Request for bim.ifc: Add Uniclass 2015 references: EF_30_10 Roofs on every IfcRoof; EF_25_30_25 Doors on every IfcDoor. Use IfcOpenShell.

First a look at what the model holds.

```python
import ifcopenshell

model = ifcopenshell.open("bim.ifc")
print(model.schema)
print("classifications:", [c.Name for c in model.by_type("IfcClassification")])
for ifc_class in ("IfcDoor", "IfcRoof", "IfcStair", "IfcWall", "IfcWindow"):
    print(ifc_class, len(model.by_type(ifc_class)))
```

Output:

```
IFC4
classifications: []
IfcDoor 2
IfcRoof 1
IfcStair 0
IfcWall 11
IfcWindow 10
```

```python
import ifcopenshell
import ifcopenshell.api.classification

model = ifcopenshell.open("bim.ifc")

system = ifcopenshell.api.classification.add_classification(model, classification="Uniclass 2015")

codes = {
    "IfcRoof": ("EF_30_10", "Roofs"),
    "IfcDoor": ("EF_25_30_25", "Doors"),
}
for ifc_class, (code, name) in codes.items():
    products = model.by_type(ifc_class)
    ifcopenshell.api.classification.add_reference(
        model, products=products, classification=system, identification=code, name=name
    )
    print(code, len(products))

model.write("bim_v2.ifc")
```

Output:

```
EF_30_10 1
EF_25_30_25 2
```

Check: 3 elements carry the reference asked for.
